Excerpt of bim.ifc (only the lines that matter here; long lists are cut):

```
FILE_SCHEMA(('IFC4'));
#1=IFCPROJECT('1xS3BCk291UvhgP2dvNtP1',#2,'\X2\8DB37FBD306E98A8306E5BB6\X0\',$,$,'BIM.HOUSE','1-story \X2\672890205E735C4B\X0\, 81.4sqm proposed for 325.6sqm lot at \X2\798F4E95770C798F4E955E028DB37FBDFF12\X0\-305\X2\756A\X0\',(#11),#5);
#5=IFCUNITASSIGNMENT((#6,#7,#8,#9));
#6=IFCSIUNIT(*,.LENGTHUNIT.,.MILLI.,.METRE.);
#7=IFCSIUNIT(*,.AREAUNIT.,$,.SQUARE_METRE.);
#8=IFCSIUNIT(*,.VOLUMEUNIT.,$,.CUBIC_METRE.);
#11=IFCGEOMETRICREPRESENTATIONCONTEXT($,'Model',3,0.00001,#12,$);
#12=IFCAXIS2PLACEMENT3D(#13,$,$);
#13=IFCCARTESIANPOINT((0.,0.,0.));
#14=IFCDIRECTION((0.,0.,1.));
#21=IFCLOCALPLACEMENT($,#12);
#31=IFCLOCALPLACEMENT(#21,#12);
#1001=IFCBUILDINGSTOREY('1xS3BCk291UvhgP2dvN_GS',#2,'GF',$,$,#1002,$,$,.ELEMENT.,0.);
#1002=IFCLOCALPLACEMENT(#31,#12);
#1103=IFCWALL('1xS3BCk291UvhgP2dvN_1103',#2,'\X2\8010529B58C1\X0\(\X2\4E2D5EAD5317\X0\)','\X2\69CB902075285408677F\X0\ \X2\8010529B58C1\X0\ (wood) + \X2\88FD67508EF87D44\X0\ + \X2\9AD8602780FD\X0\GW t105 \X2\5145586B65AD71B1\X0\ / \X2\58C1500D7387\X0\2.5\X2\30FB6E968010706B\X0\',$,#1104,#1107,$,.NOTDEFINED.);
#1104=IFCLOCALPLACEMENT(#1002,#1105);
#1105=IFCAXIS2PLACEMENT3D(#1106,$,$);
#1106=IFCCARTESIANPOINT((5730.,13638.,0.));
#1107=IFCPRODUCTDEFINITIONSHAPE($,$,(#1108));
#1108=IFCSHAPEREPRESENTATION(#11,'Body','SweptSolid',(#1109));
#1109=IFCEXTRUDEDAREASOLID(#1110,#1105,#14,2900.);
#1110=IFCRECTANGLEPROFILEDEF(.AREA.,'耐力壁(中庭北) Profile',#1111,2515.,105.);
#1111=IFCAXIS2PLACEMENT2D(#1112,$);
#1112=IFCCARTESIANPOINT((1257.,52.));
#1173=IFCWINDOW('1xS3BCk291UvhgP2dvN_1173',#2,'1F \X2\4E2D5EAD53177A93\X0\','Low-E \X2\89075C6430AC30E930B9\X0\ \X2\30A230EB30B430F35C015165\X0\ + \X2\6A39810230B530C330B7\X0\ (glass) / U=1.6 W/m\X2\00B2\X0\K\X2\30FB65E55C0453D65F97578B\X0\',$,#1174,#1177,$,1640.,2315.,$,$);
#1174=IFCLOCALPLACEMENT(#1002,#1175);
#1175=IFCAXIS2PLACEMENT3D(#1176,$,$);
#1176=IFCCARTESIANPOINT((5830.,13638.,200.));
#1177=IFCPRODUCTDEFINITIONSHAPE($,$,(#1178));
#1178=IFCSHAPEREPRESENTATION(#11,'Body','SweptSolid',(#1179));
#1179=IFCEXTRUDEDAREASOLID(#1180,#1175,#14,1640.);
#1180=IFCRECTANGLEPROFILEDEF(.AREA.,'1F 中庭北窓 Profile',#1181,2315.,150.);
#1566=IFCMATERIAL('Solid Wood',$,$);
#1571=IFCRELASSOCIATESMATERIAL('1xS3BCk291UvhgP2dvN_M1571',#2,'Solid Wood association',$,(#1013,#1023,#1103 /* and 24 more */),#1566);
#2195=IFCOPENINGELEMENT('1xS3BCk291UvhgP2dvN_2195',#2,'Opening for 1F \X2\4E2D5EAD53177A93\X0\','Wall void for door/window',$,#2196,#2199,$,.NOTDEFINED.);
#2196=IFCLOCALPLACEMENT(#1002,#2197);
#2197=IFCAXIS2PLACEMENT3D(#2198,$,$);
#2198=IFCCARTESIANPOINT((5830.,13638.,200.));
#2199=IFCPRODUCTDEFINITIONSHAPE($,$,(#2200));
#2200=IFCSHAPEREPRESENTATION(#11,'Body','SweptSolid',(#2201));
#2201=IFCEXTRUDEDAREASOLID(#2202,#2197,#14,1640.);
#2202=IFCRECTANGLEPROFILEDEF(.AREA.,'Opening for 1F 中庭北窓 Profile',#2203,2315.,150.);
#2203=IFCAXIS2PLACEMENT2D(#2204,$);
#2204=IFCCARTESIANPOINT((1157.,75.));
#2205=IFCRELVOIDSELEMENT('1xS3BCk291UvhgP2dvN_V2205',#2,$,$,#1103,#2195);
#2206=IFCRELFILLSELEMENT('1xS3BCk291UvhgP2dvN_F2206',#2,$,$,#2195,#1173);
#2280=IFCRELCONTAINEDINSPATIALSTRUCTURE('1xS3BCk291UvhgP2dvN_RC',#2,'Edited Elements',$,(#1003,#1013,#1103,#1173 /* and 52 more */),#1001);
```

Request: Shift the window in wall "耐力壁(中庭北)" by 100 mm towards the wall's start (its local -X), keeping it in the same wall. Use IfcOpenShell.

```python
import ifcopenshell
import ifcopenshell.api.geometry
import ifcopenshell.util.placement
import ifcopenshell.util.unit

model = ifcopenshell.open("bim.ifc")
unit_scale = ifcopenshell.util.unit.calculate_unit_scale(model)

window = model.by_id(1173)
opening = window.FillsVoids[0].RelatingOpeningElement
wall = opening.VoidsElements[0].RelatingBuildingElement

wall_matrix = ifcopenshell.util.placement.get_local_placement(wall.ObjectPlacement)
shift = wall_matrix[:3, 0] * -0.1 / unit_scale
before = ifcopenshell.util.placement.get_local_placement(window.ObjectPlacement)[:3, 3].copy()

# The window is not placed relative to its opening, so move both.
for product in (opening, window):
    matrix = ifcopenshell.util.placement.get_local_placement(product.ObjectPlacement)
    matrix[:3, 3] += shift
    ifcopenshell.api.geometry.edit_object_placement(model, product=product, matrix=matrix, is_si=False)

after = ifcopenshell.util.placement.get_local_placement(window.ObjectPlacement)[:3, 3]
print("window moved by", (after - before).round(3) + 0.0)

model.write("bim-out.ifc")
```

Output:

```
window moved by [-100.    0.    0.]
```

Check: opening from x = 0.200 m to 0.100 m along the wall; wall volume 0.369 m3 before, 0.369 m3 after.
